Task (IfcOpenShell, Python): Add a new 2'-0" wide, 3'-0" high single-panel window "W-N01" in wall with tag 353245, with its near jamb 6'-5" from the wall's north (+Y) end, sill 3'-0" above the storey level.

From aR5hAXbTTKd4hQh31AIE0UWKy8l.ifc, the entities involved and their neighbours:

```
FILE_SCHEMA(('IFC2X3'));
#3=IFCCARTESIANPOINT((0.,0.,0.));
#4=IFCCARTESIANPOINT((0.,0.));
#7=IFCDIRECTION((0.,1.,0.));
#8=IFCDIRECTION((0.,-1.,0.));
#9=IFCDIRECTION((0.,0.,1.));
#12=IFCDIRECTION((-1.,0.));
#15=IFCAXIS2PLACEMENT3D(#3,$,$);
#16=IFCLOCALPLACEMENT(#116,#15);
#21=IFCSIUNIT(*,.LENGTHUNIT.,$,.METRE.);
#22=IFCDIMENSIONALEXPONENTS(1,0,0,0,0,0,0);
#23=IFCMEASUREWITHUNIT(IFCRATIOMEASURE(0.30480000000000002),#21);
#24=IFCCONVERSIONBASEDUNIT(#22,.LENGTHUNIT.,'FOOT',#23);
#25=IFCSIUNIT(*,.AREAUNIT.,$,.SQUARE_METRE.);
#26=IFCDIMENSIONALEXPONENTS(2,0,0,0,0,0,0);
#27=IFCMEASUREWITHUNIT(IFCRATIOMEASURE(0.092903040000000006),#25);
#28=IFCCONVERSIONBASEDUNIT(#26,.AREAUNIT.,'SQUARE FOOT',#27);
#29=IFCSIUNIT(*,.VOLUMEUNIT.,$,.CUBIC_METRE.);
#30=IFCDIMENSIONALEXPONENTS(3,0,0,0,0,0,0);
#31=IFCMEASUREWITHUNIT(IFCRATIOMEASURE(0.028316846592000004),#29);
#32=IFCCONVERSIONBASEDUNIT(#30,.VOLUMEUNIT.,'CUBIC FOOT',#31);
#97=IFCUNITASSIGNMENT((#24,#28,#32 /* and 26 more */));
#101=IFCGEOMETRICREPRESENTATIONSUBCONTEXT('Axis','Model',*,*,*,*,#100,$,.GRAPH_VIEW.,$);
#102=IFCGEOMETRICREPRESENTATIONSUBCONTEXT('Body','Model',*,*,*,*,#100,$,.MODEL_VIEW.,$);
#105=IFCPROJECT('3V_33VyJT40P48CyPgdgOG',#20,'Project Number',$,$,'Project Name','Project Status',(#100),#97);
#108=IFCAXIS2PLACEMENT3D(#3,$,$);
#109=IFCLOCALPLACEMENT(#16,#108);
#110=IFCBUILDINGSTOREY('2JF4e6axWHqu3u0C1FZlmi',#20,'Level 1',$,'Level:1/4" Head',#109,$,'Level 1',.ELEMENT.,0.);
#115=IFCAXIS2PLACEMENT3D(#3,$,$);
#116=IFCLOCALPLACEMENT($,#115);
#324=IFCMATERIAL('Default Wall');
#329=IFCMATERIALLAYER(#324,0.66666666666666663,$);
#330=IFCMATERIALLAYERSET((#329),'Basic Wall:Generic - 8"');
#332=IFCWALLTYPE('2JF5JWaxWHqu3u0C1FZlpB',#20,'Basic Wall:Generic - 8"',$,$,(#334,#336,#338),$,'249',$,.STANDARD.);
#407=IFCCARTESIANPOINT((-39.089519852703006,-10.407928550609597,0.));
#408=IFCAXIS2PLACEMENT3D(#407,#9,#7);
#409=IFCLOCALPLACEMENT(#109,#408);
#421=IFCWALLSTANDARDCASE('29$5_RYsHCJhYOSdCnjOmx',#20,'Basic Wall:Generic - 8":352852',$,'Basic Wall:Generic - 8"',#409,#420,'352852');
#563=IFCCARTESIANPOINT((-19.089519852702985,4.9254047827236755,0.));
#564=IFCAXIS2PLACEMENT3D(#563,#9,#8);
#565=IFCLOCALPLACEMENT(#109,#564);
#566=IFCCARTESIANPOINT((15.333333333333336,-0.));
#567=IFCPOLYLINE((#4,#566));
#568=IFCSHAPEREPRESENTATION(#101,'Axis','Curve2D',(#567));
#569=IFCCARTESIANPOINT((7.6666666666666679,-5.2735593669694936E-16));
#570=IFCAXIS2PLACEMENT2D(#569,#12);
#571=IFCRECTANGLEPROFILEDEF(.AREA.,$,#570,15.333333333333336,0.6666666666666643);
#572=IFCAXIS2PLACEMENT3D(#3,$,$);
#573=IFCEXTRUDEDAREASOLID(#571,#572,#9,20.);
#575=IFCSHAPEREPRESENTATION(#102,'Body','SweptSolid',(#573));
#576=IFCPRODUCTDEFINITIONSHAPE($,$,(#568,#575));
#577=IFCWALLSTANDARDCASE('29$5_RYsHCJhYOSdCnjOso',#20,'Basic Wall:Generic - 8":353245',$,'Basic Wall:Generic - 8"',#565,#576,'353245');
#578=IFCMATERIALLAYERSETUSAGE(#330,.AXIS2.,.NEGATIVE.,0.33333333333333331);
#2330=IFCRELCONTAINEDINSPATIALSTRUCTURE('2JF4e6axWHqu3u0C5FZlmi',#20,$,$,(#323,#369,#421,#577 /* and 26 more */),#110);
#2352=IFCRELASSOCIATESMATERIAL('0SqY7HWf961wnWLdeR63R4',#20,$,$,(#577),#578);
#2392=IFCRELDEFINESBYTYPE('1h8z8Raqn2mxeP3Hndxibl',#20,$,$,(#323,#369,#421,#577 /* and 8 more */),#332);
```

```python
import numpy as np
import ifcopenshell
import ifcopenshell.api.feature
import ifcopenshell.api.geometry
import ifcopenshell.api.root
import ifcopenshell.api.spatial
import ifcopenshell.api.type
import ifcopenshell.geom
import ifcopenshell.util.element
import ifcopenshell.util.placement
import ifcopenshell.util.representation
import ifcopenshell.util.shape
import ifcopenshell.util.unit

model = ifcopenshell.open("aR5hAXbTTKd4hQh31AIE0UWKy8l.ifc")
unit_scale = ifcopenshell.util.unit.calculate_unit_scale(model)
settings = ifcopenshell.geom.settings()


def volume(element):
    """Net volume in cubic metres, openings subtracted."""
    shape = ifcopenshell.geom.create_shape(settings, element)
    return ifcopenshell.util.shape.get_volume(shape.geometry)


wall = model.by_guid("29$5_RYsHCJhYOSdCnjOso")
storey = ifcopenshell.util.element.get_container(wall, ifc_class="IfcBuildingStorey")
context = ifcopenshell.util.representation.get_context(model, "Model", "Body", "MODEL_VIEW")
before = volume(wall)

width, height, from_end, sill = 0.6096, 0.9144, 1.9558, 0.9144  # metres

# The wall runs along its own X axis, and the end named is its -X end.
wall_shape = ifcopenshell.geom.create_shape(settings, wall)
x, y, z = ifcopenshell.util.shape.get_vertices(wall_shape.geometry).T
start = x.min() + from_end
face, thickness = float(y.min()), float(y.max() - y.min())
wall_matrix = ifcopenshell.util.placement.get_local_placement(wall.ObjectPlacement)
level = ifcopenshell.util.placement.get_local_placement(storey.ObjectPlacement)[2, 3]


def in_wall(x, y):
    """Placement at x, y metres in the wall's axes, at sill height."""
    matrix = wall_matrix.copy()
    matrix[:, 3] = wall_matrix @ np.array([x / unit_scale, y / unit_scale, 0.0, 1.0])
    matrix[2, 3] = level + sill / unit_scale
    return matrix


# Opening: a box that overshoots both wall faces by 50 mm.
opening = ifcopenshell.api.root.create_entity(model, ifc_class="IfcOpeningElement")
box = ifcopenshell.api.geometry.add_wall_representation(
    model, context=context, length=width, height=height, thickness=thickness + 0.1
)
ifcopenshell.api.geometry.assign_representation(model, product=opening, representation=box)
ifcopenshell.api.geometry.edit_object_placement(model, product=opening, matrix=in_wall(start, face - 0.05), is_si=False)
ifcopenshell.api.feature.add_feature(model, feature=opening, element=wall)

window = ifcopenshell.api.root.create_entity(model, ifc_class="IfcWindow", name="W-N01")
window.OverallWidth, window.OverallHeight = width / unit_scale, height / unit_scale
body = ifcopenshell.api.geometry.add_window_representation(
    model,
    context=context,
    overall_width=window.OverallWidth,
    overall_height=window.OverallHeight,
    partition_type="SINGLE_PANEL",
)
ifcopenshell.api.geometry.assign_representation(model, product=window, representation=body)
ifcopenshell.api.spatial.assign_container(model, products=[window], relating_structure=storey)
fills = ifcopenshell.api.feature.add_filling(model, opening=opening, element=window)
fills.OwnerHistory = window.OwnerHistory  # required in IFC2X3

# IFC2X3 keeps the operation on the window style.
style = ifcopenshell.api.root.create_entity(model, ifc_class="IfcWindowStyle", name="W-N01")
style.OperationType, style.ConstructionType = "SINGLE_PANEL", "NOTDEFINED"
style.ParameterTakesPrecedence = style.Sizeable = False
ifcopenshell.api.type.assign_type(model, related_objects=[window], relating_type=style)

# Centre the window in the wall's thickness.
ifcopenshell.api.geometry.edit_object_placement(model, product=window, matrix=in_wall(start, face), is_si=False)
window_shape = ifcopenshell.geom.create_shape(settings, window)
depth = ifcopenshell.util.shape.get_vertices(window_shape.geometry)[:, 1]
offset = face + thickness / 2 - (depth.min() + depth.max()) / 2
ifcopenshell.api.geometry.edit_object_placement(model, product=window, matrix=in_wall(start, offset), is_si=False)

after = volume(wall)

print(f"wall volume {before:.3f} -> {after:.3f} m3")

model.write("aR5hAXbTTKd4hQh31AIE0UWKy8l_v2.ifc")
```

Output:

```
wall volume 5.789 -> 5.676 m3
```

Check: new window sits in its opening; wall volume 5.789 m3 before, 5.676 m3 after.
